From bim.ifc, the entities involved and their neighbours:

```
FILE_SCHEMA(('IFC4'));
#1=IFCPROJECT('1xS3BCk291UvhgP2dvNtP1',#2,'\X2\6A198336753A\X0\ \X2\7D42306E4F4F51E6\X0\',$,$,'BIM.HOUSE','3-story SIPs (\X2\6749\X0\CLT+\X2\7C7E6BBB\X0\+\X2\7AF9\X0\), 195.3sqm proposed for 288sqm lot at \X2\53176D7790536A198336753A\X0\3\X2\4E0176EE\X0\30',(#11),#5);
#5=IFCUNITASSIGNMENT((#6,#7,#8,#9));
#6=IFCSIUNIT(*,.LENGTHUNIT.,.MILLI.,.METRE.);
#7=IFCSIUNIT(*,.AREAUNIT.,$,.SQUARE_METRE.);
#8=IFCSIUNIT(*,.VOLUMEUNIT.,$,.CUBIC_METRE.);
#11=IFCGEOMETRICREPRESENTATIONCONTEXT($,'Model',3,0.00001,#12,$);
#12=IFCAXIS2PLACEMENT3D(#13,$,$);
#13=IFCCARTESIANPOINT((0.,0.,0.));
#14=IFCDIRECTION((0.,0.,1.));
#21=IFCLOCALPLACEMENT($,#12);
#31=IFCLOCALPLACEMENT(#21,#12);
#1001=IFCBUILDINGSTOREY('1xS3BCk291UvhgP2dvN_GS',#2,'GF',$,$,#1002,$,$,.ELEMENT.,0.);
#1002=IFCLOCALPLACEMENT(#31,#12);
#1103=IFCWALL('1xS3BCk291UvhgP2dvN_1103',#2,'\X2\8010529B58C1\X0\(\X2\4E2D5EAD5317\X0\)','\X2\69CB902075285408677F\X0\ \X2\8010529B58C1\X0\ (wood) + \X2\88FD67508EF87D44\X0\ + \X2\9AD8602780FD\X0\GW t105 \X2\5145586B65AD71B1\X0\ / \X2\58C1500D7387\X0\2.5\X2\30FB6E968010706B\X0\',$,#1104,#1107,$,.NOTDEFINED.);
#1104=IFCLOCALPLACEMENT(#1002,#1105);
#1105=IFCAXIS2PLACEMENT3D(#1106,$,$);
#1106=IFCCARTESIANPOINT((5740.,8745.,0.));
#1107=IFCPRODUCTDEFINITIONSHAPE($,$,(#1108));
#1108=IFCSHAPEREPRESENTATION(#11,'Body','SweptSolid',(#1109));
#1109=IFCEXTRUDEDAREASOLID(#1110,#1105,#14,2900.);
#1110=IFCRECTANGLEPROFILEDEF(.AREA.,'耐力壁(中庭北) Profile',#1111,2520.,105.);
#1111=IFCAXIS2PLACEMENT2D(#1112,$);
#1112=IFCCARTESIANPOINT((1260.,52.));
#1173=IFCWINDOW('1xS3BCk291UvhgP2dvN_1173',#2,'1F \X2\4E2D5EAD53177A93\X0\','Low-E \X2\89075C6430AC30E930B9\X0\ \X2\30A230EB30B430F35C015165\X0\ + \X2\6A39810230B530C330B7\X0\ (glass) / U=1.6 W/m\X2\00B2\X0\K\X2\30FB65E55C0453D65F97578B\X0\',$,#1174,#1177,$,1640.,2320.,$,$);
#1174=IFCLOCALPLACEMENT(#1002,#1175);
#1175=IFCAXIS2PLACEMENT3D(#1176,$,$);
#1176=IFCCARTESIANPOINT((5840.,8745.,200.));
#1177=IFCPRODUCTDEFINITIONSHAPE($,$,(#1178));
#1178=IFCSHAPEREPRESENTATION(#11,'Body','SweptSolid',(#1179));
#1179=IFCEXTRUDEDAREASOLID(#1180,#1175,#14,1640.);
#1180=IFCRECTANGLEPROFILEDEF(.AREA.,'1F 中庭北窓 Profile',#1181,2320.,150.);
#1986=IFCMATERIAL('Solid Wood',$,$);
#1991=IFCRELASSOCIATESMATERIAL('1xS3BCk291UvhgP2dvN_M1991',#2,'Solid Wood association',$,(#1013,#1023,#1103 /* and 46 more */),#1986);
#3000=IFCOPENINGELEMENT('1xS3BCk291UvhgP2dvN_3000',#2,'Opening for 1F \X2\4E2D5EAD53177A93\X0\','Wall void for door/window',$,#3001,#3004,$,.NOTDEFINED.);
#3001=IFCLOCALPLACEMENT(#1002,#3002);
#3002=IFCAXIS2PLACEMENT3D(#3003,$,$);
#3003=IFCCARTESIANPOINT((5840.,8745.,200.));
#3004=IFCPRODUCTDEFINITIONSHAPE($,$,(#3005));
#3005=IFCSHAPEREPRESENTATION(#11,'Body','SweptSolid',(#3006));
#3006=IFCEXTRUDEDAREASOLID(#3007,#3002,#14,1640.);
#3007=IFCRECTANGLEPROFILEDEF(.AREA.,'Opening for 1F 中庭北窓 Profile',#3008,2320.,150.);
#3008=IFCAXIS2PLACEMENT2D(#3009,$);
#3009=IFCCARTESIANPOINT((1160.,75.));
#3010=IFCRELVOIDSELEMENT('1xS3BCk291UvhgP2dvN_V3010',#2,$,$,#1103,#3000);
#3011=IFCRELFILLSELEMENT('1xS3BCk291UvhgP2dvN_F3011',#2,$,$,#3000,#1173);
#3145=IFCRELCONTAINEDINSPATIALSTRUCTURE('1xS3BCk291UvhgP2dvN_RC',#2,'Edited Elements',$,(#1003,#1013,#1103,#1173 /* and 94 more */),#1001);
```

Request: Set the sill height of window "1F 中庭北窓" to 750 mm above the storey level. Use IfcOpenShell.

```python
import numpy as np
import ifcopenshell
import ifcopenshell.api.geometry
import ifcopenshell.geom
import ifcopenshell.util.element
import ifcopenshell.util.placement
import ifcopenshell.util.shape
import ifcopenshell.util.unit

model = ifcopenshell.open("bim.ifc")
unit_scale = ifcopenshell.util.unit.calculate_unit_scale(model)

window = model.by_guid("1xS3BCk291UvhgP2dvN_1173")
opening = window.FillsVoids[0].RelatingOpeningElement
storey = ifcopenshell.util.element.get_container(window, ifc_class="IfcBuildingStorey")
level = ifcopenshell.util.placement.get_local_placement(storey.ObjectPlacement)[2, 3]

# The opening's origin need not be at the sill, so measure its lowest point.
shape = ifcopenshell.geom.create_shape(ifcopenshell.geom.settings(), opening)
bottom = ifcopenshell.util.shape.get_shape_bottom_elevation(shape, shape.geometry) / unit_scale
dz = level + 0.75 / unit_scale - bottom

shift = np.array([0.0, 0.0, dz])
# The window is not placed relative to its opening, so move both.
for product in (opening, window):
    matrix = ifcopenshell.util.placement.get_local_placement(product.ObjectPlacement)
    matrix[:3, 3] += shift
    ifcopenshell.api.geometry.edit_object_placement(model, product=product, matrix=matrix, is_si=False)

print(f"moved by {dz * unit_scale:+.3f} m")

model.write("bim_v2.ifc")
```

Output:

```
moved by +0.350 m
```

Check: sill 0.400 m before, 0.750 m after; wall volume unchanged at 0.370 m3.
